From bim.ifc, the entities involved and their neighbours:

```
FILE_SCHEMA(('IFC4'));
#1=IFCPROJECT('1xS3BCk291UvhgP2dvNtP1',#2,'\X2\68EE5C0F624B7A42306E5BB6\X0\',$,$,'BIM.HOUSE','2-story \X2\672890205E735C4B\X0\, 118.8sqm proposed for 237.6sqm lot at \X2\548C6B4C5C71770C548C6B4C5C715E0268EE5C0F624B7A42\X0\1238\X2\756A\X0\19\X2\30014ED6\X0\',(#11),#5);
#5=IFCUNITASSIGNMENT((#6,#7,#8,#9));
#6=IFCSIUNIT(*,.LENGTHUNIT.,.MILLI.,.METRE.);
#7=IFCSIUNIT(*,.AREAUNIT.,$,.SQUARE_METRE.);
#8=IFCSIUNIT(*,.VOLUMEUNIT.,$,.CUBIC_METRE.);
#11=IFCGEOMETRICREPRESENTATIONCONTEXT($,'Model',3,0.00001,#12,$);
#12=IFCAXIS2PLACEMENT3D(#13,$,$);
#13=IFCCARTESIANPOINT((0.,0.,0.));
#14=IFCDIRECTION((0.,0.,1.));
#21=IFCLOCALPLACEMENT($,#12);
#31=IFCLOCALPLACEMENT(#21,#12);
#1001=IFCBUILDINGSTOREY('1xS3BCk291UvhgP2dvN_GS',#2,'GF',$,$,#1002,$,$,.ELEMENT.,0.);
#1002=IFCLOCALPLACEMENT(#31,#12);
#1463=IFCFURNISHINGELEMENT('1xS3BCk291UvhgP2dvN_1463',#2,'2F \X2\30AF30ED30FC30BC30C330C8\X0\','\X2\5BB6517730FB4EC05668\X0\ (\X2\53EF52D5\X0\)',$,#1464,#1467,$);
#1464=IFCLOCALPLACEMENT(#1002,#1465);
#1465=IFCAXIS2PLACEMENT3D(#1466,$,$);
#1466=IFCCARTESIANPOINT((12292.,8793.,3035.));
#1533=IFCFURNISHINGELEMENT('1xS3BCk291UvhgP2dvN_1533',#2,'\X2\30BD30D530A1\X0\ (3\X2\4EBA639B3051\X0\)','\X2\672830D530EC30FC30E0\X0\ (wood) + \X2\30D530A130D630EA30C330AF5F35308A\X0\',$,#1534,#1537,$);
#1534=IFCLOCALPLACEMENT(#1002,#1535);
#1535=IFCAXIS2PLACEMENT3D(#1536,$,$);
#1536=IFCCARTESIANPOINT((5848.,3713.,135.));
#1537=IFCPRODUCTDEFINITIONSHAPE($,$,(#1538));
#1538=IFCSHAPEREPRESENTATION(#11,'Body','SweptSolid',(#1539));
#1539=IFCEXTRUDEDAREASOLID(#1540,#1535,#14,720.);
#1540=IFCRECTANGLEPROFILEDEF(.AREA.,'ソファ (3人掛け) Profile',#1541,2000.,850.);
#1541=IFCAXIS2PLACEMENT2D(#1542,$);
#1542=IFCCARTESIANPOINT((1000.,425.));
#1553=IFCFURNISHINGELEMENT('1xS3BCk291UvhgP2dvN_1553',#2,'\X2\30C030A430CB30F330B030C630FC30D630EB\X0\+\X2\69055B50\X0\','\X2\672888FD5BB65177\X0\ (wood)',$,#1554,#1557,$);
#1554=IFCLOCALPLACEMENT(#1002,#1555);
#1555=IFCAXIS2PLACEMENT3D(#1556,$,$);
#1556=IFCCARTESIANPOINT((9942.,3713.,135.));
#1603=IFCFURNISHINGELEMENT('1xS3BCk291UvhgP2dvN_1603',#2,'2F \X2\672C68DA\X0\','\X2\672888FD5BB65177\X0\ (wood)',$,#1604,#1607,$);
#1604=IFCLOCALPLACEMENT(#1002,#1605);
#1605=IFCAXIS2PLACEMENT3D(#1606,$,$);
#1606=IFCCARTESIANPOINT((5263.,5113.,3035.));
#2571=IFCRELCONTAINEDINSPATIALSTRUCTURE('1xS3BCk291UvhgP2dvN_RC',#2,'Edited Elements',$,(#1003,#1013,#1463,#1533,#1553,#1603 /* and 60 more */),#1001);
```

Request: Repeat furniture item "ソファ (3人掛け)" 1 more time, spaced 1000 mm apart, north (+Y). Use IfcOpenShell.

```python
import numpy as np
import ifcopenshell
import ifcopenshell.api.geometry
import ifcopenshell.api.root
import ifcopenshell.util.element
import ifcopenshell.util.placement

model = ifcopenshell.open("bim.ifc")


def reuse_history(source, copy):
    """copy_class also copies each property set's owner history, people and application; keep the originals."""
    for rel in copy.IsDefinedBy:
        if rel.is_a("IfcRelDefinesByProperties") and (history := rel.RelatingPropertyDefinition.OwnerHistory):
            rel.RelatingPropertyDefinition.OwnerHistory = source.OwnerHistory
            ifcopenshell.util.element.remove_deep2(model, history)


source = model.by_id(1533)
base = ifcopenshell.util.placement.get_local_placement(source.ObjectPlacement)
step = np.array([0.0, 1.0, 0.0]) * 1000.0

for i in range(1, 2):
    copy = ifcopenshell.api.root.copy_class(model, product=source)
    copy.Representation = ifcopenshell.util.element.copy_deep(
        model, source.Representation, exclude=["IfcGeometricRepresentationContext", "IfcRepresentationMap"]
    )
    reuse_history(source, copy)
    matrix = base.copy()
    matrix[:3, 3] += i * step
    print("added at", matrix[:3, 3].round(3) + 0.0)
    ifcopenshell.api.geometry.edit_object_placement(model, product=copy, matrix=matrix, is_si=False)

model.write("bim_v2.ifc")
```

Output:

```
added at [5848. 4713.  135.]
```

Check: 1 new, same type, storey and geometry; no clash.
